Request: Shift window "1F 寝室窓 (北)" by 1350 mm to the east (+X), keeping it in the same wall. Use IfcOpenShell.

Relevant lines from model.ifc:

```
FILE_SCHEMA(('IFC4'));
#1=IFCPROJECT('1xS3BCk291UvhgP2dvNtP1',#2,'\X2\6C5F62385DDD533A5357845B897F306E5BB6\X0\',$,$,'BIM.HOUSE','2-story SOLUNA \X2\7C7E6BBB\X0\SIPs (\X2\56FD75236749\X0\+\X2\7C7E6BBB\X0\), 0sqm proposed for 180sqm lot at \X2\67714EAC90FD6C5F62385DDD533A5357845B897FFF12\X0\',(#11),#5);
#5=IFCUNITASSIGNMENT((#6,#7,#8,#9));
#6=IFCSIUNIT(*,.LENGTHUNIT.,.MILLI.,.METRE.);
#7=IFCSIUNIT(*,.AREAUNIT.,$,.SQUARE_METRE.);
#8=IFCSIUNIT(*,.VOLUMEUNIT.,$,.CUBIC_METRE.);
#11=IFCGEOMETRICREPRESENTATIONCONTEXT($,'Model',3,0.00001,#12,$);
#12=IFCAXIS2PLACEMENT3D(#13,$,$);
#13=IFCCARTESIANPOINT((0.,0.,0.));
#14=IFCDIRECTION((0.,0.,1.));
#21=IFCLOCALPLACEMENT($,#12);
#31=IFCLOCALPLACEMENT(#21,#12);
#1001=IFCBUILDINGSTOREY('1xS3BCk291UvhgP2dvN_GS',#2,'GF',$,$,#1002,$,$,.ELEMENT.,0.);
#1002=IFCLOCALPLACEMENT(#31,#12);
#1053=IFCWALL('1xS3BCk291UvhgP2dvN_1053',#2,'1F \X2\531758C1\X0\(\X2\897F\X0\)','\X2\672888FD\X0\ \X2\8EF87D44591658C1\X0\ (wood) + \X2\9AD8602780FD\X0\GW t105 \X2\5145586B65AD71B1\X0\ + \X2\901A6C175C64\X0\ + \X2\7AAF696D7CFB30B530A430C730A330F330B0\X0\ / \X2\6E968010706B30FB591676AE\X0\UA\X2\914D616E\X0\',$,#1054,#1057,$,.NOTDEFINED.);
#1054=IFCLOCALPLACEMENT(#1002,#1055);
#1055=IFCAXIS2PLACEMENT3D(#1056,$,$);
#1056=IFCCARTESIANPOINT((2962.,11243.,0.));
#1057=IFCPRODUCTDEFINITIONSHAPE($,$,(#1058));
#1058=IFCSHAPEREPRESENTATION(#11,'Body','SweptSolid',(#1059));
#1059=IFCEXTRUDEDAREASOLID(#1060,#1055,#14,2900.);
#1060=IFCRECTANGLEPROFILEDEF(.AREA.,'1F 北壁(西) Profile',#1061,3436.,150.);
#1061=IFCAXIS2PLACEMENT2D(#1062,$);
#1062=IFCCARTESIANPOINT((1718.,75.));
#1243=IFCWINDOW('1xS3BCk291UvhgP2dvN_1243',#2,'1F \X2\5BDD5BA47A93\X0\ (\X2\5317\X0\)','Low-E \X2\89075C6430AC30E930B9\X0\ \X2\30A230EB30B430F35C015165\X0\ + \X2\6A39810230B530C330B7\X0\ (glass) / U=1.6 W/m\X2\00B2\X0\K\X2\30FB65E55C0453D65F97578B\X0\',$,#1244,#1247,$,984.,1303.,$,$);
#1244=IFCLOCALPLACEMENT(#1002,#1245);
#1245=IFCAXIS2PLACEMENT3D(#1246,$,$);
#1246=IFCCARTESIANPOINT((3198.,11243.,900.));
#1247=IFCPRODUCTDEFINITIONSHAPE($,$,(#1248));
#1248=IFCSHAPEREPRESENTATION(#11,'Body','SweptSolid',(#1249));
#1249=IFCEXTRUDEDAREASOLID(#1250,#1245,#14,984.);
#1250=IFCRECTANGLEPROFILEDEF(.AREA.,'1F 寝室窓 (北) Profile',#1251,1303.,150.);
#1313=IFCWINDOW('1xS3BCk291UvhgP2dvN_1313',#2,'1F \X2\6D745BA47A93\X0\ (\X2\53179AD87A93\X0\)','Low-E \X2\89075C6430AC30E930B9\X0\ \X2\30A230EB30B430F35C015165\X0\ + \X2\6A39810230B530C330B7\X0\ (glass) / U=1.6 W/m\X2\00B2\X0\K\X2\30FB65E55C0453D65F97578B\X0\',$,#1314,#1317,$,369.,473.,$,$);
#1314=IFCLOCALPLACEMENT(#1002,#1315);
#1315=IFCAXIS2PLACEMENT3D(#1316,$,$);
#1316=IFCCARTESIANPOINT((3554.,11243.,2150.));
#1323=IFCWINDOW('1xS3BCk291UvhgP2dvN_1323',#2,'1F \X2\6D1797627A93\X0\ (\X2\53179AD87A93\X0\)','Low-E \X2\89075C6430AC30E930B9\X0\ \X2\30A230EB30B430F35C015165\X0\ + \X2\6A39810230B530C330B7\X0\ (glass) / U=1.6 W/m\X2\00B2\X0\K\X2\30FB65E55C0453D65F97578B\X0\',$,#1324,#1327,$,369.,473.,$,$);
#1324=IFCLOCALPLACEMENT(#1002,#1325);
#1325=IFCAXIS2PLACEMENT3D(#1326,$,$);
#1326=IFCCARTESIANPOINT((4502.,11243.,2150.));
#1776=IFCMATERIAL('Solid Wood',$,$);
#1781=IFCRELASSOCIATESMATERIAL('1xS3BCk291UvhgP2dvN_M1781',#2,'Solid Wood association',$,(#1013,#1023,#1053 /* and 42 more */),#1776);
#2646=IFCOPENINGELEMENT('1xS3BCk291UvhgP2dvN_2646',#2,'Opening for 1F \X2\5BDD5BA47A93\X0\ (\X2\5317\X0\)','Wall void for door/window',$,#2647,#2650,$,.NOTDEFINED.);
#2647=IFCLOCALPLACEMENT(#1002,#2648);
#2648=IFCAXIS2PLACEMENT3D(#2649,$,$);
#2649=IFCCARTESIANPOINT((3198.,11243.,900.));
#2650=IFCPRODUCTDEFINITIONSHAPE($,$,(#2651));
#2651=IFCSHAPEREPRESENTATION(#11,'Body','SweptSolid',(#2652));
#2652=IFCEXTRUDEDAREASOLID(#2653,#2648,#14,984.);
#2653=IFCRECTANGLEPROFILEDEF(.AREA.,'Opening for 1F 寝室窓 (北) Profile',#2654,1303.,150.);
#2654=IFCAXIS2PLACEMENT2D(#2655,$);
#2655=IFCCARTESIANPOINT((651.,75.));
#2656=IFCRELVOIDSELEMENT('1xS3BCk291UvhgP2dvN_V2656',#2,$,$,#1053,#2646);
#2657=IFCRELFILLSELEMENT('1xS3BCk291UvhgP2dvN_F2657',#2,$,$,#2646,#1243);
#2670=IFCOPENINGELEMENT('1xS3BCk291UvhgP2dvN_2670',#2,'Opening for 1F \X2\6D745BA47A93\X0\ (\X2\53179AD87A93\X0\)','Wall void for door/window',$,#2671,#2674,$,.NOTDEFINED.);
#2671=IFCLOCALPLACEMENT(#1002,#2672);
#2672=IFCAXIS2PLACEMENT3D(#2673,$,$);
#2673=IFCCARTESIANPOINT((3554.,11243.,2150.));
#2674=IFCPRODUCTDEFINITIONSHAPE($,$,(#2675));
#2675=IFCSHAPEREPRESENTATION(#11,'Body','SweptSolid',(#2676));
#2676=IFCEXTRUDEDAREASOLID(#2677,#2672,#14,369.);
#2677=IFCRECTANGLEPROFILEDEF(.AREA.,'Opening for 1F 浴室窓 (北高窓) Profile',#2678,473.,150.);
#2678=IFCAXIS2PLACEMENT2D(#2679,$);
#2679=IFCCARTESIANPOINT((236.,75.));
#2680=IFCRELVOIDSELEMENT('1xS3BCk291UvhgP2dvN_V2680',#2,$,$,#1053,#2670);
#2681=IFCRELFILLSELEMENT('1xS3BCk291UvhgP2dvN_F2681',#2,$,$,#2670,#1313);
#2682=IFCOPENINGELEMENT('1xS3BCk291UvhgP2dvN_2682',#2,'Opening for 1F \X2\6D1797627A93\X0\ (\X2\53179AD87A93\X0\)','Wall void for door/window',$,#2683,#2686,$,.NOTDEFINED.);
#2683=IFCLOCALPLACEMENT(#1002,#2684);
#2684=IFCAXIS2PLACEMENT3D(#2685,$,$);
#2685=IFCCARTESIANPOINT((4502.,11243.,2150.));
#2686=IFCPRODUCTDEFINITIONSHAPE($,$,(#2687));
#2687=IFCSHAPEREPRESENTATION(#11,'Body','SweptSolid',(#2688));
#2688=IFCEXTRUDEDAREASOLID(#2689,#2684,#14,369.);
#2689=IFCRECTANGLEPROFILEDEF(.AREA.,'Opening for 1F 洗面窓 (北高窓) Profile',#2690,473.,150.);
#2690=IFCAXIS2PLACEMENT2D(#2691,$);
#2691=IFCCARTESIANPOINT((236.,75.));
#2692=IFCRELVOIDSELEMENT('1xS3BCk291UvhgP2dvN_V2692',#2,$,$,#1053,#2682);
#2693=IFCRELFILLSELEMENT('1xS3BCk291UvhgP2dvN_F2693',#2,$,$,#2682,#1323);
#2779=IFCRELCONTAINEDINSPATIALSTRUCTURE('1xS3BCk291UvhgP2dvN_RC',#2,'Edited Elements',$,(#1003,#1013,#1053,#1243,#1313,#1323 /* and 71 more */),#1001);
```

```python
import ifcopenshell
import ifcopenshell.api.geometry
import ifcopenshell.util.placement
import ifcopenshell.util.unit

model = ifcopenshell.open("model.ifc")
unit_scale = ifcopenshell.util.unit.calculate_unit_scale(model)

window = model.by_guid("1xS3BCk291UvhgP2dvN_1243")
opening = window.FillsVoids[0].RelatingOpeningElement
wall = opening.VoidsElements[0].RelatingBuildingElement

wall_matrix = ifcopenshell.util.placement.get_local_placement(wall.ObjectPlacement)
shift = wall_matrix[:3, 0] * 1.35 / unit_scale
before = ifcopenshell.util.placement.get_local_placement(window.ObjectPlacement)[:3, 3].copy()

# The window is not placed relative to its opening, so move both.
for product in (opening, window):
    matrix = ifcopenshell.util.placement.get_local_placement(product.ObjectPlacement)
    matrix[:3, 3] += shift
    ifcopenshell.api.geometry.edit_object_placement(model, product=product, matrix=matrix, is_si=False)

after = ifcopenshell.util.placement.get_local_placement(window.ObjectPlacement)[:3, 3]
print("window moved by", (after - before).round(3) + 0.0)

model.write("model_updated.ifc")
```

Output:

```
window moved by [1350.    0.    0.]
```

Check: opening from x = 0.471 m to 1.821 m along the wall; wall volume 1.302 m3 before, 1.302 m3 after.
